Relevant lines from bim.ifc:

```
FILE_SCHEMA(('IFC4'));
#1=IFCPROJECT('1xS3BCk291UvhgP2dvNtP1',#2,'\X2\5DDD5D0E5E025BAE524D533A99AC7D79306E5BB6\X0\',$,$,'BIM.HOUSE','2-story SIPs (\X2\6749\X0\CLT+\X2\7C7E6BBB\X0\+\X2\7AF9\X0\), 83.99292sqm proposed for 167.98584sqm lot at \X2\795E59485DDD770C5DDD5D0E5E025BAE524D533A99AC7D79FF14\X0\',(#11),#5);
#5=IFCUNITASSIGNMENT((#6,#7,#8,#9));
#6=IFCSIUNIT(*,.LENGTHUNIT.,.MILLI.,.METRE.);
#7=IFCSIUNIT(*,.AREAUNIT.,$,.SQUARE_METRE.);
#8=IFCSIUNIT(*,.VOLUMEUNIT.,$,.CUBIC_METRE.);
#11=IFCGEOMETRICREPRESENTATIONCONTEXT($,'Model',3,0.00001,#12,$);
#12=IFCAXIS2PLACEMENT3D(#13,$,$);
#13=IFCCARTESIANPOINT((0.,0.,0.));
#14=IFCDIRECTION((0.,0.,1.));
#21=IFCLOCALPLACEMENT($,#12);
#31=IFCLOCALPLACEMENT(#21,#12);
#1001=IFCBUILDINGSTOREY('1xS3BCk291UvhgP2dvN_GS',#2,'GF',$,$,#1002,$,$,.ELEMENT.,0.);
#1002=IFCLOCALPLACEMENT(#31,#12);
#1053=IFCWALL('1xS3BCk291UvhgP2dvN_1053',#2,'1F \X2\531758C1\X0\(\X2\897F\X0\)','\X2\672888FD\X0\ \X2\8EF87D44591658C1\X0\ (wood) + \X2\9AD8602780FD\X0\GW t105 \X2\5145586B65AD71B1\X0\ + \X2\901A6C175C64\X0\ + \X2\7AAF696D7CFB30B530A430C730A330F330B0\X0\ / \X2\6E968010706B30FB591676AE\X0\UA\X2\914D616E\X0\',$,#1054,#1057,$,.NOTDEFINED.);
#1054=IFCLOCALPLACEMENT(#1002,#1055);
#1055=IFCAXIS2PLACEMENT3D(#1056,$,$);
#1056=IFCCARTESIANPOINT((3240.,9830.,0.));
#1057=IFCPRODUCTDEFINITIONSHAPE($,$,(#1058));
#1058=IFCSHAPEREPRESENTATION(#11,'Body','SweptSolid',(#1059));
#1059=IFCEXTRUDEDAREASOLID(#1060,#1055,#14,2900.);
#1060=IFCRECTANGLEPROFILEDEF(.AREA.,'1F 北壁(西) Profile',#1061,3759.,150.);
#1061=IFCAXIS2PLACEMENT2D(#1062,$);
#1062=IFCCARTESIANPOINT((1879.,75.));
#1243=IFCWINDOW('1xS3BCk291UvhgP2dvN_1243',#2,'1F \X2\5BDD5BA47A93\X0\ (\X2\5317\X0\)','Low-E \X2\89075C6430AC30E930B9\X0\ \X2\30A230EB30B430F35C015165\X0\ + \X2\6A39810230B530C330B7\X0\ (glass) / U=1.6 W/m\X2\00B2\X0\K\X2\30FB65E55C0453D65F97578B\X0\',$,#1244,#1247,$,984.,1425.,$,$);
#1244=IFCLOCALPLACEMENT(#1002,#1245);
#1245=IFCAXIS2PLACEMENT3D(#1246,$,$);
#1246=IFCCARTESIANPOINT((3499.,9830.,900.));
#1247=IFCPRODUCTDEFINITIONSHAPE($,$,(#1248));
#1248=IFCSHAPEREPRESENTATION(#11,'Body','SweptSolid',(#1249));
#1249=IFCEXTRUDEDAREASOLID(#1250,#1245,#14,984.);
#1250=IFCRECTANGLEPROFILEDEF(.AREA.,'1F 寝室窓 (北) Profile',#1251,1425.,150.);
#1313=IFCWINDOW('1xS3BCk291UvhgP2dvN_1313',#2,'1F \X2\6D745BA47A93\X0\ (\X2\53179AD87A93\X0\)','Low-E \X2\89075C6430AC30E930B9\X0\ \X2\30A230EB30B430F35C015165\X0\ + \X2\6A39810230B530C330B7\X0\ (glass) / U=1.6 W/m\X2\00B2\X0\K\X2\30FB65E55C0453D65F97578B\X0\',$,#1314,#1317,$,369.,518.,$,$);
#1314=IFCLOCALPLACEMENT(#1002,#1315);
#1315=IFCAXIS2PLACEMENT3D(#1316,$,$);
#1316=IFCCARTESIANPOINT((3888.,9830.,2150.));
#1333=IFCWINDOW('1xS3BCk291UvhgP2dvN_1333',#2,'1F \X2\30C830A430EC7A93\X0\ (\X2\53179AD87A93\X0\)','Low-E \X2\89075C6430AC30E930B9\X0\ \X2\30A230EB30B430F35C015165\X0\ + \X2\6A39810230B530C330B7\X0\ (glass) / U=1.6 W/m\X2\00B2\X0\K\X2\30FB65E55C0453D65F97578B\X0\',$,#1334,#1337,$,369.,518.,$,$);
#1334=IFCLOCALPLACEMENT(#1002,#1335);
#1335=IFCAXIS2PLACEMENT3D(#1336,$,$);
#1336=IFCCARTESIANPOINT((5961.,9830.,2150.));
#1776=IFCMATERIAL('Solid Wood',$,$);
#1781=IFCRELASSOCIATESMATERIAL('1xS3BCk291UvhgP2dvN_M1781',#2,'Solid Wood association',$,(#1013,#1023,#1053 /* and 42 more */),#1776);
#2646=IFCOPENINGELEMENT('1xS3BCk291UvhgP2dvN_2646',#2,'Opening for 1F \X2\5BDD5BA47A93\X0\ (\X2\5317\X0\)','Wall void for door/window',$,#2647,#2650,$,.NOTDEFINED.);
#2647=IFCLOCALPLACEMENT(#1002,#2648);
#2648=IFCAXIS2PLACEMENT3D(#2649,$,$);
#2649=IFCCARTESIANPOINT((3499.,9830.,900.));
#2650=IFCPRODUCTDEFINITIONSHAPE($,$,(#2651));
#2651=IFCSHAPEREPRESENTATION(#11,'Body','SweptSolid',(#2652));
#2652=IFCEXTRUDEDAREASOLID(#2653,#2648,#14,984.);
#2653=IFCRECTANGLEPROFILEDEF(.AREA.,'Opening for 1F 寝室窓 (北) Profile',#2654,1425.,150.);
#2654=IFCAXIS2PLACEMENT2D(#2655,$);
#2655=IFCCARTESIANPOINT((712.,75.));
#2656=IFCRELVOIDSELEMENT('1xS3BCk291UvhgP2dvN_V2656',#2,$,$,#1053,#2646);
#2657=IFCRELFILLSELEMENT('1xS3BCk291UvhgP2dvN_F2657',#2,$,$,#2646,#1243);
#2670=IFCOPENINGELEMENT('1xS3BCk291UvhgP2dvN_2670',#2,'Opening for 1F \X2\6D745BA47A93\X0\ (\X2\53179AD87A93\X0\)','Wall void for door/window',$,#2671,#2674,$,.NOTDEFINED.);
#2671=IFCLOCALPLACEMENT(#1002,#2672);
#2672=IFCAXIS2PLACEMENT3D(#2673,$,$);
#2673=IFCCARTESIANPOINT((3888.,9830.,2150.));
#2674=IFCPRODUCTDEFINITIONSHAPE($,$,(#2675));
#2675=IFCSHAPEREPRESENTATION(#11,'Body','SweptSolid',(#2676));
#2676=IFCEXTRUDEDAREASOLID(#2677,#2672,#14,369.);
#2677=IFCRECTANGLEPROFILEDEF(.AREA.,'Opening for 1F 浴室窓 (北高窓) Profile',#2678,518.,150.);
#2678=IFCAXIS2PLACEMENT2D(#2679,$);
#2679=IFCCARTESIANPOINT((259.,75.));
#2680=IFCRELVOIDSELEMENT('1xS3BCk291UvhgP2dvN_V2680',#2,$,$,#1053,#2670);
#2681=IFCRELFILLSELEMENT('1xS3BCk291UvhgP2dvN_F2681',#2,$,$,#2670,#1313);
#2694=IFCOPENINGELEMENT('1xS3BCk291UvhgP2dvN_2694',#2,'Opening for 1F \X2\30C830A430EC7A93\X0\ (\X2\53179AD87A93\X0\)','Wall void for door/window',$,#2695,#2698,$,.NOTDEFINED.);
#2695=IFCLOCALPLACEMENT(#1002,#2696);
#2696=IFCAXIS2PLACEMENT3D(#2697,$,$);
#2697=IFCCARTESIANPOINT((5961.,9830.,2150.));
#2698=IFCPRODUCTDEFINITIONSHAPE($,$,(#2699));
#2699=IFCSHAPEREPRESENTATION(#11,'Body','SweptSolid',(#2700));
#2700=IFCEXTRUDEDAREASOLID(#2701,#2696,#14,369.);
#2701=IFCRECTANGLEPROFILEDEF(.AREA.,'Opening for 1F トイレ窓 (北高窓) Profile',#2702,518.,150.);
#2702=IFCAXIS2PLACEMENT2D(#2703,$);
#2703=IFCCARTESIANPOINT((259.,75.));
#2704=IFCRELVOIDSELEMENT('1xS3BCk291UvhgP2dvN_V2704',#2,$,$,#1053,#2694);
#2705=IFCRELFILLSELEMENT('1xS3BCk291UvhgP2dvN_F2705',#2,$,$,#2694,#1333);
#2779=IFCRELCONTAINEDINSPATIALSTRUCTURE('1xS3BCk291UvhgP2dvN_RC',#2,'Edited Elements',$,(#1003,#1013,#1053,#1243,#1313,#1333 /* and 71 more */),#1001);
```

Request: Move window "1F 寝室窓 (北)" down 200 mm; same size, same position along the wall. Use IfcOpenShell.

```python
import numpy as np
import ifcopenshell
import ifcopenshell.api.geometry
import ifcopenshell.util.placement
import ifcopenshell.util.unit

model = ifcopenshell.open("bim.ifc")
unit_scale = ifcopenshell.util.unit.calculate_unit_scale(model)

window = model.by_guid("1xS3BCk291UvhgP2dvN_1243")
opening = window.FillsVoids[0].RelatingOpeningElement
dz = -0.2 / unit_scale

shift = np.array([0.0, 0.0, dz])
# The window is not placed relative to its opening, so move both.
for product in (opening, window):
    matrix = ifcopenshell.util.placement.get_local_placement(product.ObjectPlacement)
    matrix[:3, 3] += shift
    ifcopenshell.api.geometry.edit_object_placement(model, product=product, matrix=matrix, is_si=False)

print(f"moved by {dz * unit_scale:+.3f} m")

model.write("bim_edited.ifc")
```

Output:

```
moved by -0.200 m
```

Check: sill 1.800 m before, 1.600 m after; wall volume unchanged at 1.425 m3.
